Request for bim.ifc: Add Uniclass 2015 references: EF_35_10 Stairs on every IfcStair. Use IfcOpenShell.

First a look at what the model holds.

```python
import ifcopenshell

model = ifcopenshell.open("bim.ifc")
print(model.schema)
print("classifications:", [c.Name for c in model.by_type("IfcClassification")])
for ifc_class in ("IfcDoor", "IfcRoof", "IfcStair", "IfcWall", "IfcWindow"):
    print(ifc_class, len(model.by_type(ifc_class)))
```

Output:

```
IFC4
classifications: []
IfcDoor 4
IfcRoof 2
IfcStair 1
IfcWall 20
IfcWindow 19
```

```python
import ifcopenshell
import ifcopenshell.api.classification

model = ifcopenshell.open("bim.ifc")

system = ifcopenshell.api.classification.add_classification(model, classification="Uniclass 2015")

codes = {
    "IfcStair": ("EF_35_10", "Stairs"),
}
for ifc_class, (code, name) in codes.items():
    products = model.by_type(ifc_class)
    ifcopenshell.api.classification.add_reference(
        model, products=products, classification=system, identification=code, name=name
    )
    print(code, len(products))

model.write("bim_v2.ifc")
```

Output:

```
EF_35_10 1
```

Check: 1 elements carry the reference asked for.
